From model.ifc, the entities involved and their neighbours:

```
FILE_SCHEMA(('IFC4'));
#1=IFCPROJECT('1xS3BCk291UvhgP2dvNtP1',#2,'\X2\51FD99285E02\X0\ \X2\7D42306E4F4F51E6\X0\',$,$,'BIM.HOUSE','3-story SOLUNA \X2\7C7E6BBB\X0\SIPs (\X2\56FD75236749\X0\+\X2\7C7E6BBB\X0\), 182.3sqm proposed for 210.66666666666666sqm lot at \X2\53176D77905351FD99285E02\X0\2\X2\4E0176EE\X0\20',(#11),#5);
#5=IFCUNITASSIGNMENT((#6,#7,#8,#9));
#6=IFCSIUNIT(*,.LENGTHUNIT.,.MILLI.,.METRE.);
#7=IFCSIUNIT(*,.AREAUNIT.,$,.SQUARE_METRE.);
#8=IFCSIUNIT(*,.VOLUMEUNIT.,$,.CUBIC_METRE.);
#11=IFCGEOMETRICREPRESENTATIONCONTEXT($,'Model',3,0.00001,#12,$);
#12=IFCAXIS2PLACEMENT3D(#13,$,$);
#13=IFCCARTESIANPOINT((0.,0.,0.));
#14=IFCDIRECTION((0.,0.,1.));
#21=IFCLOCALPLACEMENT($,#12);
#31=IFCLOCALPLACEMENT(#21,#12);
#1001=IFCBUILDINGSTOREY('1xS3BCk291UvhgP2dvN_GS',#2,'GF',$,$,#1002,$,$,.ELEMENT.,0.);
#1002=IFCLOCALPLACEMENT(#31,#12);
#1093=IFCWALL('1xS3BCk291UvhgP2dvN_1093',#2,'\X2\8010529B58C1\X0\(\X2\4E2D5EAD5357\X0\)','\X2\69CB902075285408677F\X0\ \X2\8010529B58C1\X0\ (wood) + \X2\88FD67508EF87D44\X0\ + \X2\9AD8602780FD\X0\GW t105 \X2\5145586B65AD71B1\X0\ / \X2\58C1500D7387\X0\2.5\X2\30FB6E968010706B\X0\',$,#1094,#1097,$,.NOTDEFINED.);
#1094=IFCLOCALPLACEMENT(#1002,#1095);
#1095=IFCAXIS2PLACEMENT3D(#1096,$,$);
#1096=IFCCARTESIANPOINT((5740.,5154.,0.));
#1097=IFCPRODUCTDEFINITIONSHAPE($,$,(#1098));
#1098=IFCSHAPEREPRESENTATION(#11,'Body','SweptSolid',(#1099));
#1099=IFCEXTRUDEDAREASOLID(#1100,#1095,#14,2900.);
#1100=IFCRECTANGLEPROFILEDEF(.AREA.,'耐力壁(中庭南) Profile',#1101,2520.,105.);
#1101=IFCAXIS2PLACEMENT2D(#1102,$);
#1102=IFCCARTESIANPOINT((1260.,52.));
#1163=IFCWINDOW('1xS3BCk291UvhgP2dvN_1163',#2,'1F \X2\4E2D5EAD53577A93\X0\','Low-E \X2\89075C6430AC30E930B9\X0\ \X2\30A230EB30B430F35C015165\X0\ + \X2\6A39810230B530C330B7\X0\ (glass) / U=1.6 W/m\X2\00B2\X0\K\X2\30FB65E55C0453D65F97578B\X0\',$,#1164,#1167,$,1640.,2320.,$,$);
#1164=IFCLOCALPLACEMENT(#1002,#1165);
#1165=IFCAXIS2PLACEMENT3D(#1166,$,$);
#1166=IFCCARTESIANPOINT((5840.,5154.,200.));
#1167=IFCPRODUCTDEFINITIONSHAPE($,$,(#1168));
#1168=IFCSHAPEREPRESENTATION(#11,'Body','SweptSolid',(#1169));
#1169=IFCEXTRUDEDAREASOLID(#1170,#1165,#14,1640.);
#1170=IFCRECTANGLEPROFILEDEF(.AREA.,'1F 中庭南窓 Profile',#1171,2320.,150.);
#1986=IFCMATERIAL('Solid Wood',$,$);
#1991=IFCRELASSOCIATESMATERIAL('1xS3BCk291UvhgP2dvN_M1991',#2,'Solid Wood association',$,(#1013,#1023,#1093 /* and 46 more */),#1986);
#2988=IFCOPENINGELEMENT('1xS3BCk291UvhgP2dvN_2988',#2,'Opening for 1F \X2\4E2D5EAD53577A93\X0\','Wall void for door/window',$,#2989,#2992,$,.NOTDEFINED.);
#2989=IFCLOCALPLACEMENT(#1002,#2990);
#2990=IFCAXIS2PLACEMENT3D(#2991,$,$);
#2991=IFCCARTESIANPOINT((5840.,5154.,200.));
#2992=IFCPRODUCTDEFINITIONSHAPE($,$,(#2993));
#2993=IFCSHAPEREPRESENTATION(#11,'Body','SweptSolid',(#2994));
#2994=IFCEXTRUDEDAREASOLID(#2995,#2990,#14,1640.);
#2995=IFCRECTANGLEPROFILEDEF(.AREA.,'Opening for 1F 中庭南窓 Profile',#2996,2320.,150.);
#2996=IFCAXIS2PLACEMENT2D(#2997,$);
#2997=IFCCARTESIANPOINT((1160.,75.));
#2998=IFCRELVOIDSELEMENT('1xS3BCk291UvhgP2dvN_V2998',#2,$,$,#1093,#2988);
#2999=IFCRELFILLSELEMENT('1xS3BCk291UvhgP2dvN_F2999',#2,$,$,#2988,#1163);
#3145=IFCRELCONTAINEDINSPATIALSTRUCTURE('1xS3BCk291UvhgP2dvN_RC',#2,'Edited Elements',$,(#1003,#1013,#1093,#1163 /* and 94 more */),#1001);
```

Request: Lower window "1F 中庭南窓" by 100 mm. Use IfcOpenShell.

```python
import numpy as np
import ifcopenshell
import ifcopenshell.api.geometry
import ifcopenshell.util.placement
import ifcopenshell.util.unit

model = ifcopenshell.open("model.ifc")
unit_scale = ifcopenshell.util.unit.calculate_unit_scale(model)

window = model.by_id(1163)
opening = window.FillsVoids[0].RelatingOpeningElement
dz = -100.0

shift = np.array([0.0, 0.0, dz])
# The window is not placed relative to its opening, so move both.
for product in (opening, window):
    matrix = ifcopenshell.util.placement.get_local_placement(product.ObjectPlacement)
    matrix[:3, 3] += shift
    ifcopenshell.api.geometry.edit_object_placement(model, product=product, matrix=matrix, is_si=False)

print(f"moved by {dz * unit_scale:+.3f} m")

model.write("model_updated.ifc")
```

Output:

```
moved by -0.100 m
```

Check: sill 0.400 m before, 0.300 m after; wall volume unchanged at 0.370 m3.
